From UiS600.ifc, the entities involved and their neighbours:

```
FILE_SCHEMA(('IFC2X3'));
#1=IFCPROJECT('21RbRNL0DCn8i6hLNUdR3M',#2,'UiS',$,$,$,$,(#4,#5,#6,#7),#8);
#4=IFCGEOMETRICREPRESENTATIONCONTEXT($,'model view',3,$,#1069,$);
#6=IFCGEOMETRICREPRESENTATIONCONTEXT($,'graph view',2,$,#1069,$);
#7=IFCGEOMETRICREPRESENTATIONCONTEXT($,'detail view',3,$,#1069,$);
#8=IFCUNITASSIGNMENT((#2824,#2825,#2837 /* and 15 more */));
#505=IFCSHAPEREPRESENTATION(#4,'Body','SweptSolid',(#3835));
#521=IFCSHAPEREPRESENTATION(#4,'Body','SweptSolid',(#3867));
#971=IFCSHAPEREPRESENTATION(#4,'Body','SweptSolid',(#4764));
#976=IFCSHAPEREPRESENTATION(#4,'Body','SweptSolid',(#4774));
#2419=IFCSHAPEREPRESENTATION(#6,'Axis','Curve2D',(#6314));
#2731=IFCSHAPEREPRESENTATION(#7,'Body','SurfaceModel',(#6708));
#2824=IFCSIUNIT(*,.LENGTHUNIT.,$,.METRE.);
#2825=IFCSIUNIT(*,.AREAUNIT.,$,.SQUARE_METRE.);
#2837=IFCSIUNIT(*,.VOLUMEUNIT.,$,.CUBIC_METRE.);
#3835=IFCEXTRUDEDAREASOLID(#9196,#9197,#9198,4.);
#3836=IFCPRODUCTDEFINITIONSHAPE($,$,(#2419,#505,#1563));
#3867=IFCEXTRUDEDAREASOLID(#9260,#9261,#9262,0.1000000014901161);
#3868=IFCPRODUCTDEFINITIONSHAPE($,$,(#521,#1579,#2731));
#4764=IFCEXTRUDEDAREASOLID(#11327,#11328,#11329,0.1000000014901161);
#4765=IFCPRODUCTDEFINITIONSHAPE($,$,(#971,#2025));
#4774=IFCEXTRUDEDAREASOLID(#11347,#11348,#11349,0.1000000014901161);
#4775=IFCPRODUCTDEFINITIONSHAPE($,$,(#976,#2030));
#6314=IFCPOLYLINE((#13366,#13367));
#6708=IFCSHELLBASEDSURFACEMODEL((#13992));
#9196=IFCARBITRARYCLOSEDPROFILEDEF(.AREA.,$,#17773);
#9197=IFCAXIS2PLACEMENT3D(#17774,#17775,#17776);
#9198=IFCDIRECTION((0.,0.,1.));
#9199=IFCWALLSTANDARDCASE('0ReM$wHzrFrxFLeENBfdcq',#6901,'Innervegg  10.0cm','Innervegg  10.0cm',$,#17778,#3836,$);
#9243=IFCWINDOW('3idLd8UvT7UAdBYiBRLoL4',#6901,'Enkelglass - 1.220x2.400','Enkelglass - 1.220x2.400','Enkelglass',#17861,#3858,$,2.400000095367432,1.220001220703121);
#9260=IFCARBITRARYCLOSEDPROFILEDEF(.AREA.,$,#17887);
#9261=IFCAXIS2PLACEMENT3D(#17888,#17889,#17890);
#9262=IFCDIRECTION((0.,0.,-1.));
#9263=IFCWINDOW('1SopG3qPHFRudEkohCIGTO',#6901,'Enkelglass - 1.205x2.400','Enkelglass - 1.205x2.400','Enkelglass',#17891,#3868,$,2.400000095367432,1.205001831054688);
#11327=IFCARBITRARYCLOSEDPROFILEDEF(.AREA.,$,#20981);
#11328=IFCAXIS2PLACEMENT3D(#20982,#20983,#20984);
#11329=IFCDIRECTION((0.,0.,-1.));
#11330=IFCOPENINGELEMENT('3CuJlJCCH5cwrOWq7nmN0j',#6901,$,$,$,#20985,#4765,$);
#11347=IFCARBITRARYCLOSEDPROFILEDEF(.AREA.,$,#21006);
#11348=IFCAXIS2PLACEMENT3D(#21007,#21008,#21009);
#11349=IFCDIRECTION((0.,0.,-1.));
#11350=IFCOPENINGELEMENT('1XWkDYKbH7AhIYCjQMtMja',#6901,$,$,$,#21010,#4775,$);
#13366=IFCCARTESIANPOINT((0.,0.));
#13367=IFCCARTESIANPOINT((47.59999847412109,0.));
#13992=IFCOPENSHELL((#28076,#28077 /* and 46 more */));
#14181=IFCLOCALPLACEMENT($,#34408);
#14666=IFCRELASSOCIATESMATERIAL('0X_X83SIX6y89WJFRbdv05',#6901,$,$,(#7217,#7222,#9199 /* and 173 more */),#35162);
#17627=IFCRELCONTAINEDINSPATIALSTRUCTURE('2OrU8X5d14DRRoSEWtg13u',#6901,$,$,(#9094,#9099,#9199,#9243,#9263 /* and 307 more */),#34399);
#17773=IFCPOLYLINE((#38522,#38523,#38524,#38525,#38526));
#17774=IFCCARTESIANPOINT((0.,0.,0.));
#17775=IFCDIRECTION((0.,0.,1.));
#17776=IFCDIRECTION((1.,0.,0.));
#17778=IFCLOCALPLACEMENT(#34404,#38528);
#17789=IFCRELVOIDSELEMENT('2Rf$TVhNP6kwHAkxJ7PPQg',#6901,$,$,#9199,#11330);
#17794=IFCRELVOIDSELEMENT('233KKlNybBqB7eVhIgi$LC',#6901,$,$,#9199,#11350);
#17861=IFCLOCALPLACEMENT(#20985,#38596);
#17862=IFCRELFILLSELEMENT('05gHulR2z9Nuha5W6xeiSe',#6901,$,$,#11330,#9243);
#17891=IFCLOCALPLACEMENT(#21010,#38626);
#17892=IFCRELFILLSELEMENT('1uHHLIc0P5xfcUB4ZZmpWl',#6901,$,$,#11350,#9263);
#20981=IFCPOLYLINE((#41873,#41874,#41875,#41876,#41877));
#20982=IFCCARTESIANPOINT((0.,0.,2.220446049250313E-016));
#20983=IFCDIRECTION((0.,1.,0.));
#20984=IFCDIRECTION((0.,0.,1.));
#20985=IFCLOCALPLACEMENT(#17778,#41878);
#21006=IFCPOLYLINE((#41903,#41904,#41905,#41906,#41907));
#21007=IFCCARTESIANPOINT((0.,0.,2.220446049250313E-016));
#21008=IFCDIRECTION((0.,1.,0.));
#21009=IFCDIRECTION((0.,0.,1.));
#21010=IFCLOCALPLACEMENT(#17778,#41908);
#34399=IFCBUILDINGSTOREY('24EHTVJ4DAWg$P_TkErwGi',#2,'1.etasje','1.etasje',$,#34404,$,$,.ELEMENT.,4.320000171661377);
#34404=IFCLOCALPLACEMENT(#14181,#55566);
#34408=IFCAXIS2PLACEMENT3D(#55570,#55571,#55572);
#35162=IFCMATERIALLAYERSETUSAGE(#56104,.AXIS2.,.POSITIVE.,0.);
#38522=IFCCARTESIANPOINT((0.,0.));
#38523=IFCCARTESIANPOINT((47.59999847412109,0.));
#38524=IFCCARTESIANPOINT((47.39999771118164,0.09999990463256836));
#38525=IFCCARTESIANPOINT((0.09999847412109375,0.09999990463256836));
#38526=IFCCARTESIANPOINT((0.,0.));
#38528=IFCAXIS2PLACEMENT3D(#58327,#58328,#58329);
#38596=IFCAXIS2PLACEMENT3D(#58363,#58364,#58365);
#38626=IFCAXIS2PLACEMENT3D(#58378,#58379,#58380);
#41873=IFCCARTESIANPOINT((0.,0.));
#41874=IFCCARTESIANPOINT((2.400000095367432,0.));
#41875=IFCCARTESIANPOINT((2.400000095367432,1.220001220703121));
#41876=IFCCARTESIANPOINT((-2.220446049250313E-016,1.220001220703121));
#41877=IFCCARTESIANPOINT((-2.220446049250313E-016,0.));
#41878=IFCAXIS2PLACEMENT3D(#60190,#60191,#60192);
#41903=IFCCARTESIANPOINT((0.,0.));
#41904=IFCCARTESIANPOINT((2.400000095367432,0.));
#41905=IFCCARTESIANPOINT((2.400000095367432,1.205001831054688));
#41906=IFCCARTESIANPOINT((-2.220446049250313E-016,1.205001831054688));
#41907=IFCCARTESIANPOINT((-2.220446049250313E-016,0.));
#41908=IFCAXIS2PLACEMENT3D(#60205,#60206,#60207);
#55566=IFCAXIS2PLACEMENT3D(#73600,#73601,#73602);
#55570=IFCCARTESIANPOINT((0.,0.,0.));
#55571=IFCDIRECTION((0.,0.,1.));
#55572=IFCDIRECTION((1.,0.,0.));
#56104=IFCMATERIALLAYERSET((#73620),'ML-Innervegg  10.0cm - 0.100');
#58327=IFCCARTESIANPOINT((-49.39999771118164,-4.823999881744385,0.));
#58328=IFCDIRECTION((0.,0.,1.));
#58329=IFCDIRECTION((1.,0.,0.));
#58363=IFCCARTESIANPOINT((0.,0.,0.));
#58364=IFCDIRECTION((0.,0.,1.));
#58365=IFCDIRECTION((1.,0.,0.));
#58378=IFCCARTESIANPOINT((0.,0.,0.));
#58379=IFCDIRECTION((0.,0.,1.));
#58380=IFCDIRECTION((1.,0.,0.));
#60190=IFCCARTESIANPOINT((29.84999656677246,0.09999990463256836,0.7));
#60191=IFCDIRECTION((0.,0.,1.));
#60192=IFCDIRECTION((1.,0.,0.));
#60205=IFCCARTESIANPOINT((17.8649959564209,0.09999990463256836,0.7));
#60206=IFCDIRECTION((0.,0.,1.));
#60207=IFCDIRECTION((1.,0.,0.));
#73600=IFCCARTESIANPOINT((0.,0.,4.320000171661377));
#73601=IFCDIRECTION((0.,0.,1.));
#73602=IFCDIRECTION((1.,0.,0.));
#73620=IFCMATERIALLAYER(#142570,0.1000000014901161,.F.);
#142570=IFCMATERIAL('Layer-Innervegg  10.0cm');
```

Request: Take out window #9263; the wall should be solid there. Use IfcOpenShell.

```python
import ifcopenshell
import ifcopenshell.api.feature
import ifcopenshell.api.root
import ifcopenshell.geom
import ifcopenshell.util.shape

model = ifcopenshell.open("UiS600.ifc")
settings = ifcopenshell.geom.settings()


def volume(element):
    """Net volume in cubic metres, openings subtracted."""
    shape = ifcopenshell.geom.create_shape(settings, element)
    return ifcopenshell.util.shape.get_volume(shape.geometry)


window = model.by_guid("1SopG3qPHFRudEkohCIGTO")
opening = window.FillsVoids[0].RelatingOpeningElement
wall = opening.VoidsElements[0].RelatingBuildingElement
before = volume(wall)

ifcopenshell.api.root.remove_product(model, product=window)
ifcopenshell.api.feature.remove_feature(model, feature=opening)

after = volume(wall)

print(f"wall volume {before:.3f} -> {after:.3f} m3")

model.write("UiS600_updated.ifc")
```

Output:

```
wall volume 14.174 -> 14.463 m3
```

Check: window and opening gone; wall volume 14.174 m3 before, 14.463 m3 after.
